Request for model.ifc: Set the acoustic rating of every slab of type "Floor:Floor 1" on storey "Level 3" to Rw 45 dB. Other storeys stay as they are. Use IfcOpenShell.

First a look at what the model holds.

```python
import ifcopenshell
import ifcopenshell.util.element

model = ifcopenshell.open("model.ifc")
print(model.schema)
storey = next(s for s in model.by_type("IfcBuildingStorey") if s.Name == "Level 3")
slabs = [e for e in ifcopenshell.util.element.get_decomposition(storey) if e.is_a("IfcSlab")]
seen = {}
for e in slabs:
    element_type = ifcopenshell.util.element.get_type(e)
    key = (element_type.Name if element_type != e and element_type else None, ifcopenshell.util.element.get_pset(e, "Pset_SlabCommon", "AcousticRating"))
    seen[key] = seen.get(key, 0) + 1
for (name, value), count in sorted(seen.items(), key=str):
    print(count, "x", name, "|", value)
```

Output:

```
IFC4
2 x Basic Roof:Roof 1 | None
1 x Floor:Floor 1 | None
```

```python
import ifcopenshell
import ifcopenshell.api.pset
import ifcopenshell.util.element

model = ifcopenshell.open("model.ifc")

storey = next(s for s in model.by_type("IfcBuildingStorey") if s.Name == "Level 3")
slabs = [e for e in ifcopenshell.util.element.get_decomposition(storey) if e.is_a("IfcSlab")]

count = 0
for e in slabs:
    element_type = ifcopenshell.util.element.get_type(e)
    if element_type in (None, e) or element_type.Name != "Floor:Floor 1":
        continue
    # add_pset returns the element's existing set when there is one.
    pset = ifcopenshell.api.pset.add_pset(model, product=e, name="Pset_SlabCommon")
    ifcopenshell.api.pset.edit_pset(model, pset=pset, properties={"AcousticRating": "Rw 45 dB"})
    count += 1

print(count, "slabs updated")

model.write("model-out.ifc")
```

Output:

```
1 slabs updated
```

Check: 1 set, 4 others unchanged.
